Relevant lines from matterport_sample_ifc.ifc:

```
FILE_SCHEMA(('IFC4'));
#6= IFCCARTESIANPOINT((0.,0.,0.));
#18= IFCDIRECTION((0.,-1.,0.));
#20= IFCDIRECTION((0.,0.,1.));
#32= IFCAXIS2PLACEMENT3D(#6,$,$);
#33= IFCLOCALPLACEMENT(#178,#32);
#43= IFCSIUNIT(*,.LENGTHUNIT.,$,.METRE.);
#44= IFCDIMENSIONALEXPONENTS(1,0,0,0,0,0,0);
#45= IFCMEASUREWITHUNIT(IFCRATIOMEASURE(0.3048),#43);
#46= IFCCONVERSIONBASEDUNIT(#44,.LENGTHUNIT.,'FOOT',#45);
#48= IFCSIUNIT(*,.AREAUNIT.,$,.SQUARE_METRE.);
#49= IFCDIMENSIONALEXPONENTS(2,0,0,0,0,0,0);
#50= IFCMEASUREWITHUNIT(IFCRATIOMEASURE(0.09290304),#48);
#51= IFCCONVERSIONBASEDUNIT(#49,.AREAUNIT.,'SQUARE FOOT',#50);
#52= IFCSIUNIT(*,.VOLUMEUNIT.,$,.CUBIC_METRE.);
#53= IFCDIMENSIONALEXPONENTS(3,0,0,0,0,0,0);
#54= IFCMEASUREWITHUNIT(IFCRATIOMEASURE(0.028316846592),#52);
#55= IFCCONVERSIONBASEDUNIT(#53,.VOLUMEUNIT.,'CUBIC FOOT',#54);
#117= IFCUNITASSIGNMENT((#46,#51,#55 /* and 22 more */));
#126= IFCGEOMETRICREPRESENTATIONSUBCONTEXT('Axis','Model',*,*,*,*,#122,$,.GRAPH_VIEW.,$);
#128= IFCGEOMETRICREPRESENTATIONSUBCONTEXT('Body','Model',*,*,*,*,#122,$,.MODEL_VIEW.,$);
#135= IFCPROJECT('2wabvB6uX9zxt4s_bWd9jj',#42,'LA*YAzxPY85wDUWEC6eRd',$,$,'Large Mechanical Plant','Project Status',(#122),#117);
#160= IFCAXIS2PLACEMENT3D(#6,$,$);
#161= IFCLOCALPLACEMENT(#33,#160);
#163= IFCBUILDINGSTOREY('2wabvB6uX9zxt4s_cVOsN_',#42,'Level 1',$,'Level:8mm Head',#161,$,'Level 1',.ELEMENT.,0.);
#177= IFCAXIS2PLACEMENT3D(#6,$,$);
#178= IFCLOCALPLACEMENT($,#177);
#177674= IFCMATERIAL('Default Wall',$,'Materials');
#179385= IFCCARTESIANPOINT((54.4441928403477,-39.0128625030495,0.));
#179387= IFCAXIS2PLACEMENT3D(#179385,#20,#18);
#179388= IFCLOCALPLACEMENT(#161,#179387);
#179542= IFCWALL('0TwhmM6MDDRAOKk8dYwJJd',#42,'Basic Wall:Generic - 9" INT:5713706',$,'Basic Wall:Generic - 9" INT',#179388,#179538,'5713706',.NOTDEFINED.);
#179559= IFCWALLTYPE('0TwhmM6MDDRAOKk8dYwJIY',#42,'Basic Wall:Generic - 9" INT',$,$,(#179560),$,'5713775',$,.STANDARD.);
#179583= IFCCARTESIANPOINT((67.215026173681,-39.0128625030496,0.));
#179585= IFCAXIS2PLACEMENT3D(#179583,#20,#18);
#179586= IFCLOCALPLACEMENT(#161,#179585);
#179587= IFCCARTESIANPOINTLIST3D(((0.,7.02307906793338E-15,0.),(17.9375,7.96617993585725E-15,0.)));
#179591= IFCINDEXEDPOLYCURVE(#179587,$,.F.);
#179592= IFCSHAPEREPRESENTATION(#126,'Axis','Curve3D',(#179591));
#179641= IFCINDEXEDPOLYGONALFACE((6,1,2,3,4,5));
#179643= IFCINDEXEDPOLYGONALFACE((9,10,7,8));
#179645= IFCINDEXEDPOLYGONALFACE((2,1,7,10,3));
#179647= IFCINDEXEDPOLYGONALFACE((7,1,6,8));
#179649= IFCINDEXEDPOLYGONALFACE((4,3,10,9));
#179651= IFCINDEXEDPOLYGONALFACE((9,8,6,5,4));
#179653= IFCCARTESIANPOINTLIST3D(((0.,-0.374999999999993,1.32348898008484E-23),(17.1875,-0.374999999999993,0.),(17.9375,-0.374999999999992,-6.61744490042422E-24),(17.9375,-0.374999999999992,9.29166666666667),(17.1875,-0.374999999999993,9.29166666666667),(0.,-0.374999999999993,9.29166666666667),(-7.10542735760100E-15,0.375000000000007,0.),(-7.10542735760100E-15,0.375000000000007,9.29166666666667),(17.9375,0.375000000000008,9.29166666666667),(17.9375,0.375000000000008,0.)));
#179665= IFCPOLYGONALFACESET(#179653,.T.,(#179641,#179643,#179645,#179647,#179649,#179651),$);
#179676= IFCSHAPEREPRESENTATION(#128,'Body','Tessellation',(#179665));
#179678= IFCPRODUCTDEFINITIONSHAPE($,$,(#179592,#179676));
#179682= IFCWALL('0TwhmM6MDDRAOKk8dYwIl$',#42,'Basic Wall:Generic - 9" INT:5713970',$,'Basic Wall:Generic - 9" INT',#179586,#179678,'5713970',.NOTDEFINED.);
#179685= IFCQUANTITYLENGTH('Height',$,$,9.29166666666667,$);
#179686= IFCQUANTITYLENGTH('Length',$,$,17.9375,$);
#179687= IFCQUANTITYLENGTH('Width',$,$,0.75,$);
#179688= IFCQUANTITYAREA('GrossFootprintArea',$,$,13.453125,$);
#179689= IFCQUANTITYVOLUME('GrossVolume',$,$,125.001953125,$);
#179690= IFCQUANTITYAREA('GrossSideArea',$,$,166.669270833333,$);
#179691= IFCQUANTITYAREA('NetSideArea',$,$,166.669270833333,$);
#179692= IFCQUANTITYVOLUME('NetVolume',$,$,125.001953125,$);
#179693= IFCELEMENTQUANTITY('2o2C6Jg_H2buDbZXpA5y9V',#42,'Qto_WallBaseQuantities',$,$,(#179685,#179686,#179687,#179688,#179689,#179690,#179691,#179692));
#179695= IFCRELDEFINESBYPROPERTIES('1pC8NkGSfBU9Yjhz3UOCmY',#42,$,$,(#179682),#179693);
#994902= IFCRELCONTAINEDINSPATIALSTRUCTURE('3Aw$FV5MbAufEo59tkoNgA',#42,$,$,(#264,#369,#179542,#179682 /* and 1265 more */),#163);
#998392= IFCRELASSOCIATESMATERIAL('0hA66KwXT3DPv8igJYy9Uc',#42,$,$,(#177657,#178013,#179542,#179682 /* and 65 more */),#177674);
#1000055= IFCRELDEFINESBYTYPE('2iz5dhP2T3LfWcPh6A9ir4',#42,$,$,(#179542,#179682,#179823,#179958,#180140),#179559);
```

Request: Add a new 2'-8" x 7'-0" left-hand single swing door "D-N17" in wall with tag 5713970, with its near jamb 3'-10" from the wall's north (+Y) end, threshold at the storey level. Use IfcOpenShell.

```python
import numpy as np
import ifcopenshell
import ifcopenshell.api.feature
import ifcopenshell.api.geometry
import ifcopenshell.api.pset
import ifcopenshell.api.root
import ifcopenshell.api.spatial
import ifcopenshell.geom
import ifcopenshell.util.element
import ifcopenshell.util.placement
import ifcopenshell.util.representation
import ifcopenshell.util.shape
import ifcopenshell.util.unit

model = ifcopenshell.open("matterport_sample_ifc.ifc")
unit_scale = ifcopenshell.util.unit.calculate_unit_scale(model)
area_scale = ifcopenshell.util.unit.calculate_unit_scale(model, "AREAUNIT")
volume_scale = ifcopenshell.util.unit.calculate_unit_scale(model, "VOLUMEUNIT")
settings = ifcopenshell.geom.settings()


def volume(element):
    """Net volume in cubic metres, openings subtracted."""
    shape = ifcopenshell.geom.create_shape(settings, element)
    return ifcopenshell.util.shape.get_volume(shape.geometry)


wall = model.by_guid("0TwhmM6MDDRAOKk8dYwIl$")
storey = ifcopenshell.util.element.get_container(wall, ifc_class="IfcBuildingStorey")
context = ifcopenshell.util.representation.get_context(model, "Model", "Body", "MODEL_VIEW")
before = volume(wall)

width, height, from_end, sill = 0.8128, 2.1336, 1.1684, 0.0  # metres

# The wall runs along its own X axis, and the end named is its -X end.
wall_shape = ifcopenshell.geom.create_shape(settings, wall)
x, y, z = ifcopenshell.util.shape.get_vertices(wall_shape.geometry).T
start = x.min() + from_end
face, thickness = float(y.min()), float(y.max() - y.min())
wall_matrix = ifcopenshell.util.placement.get_local_placement(wall.ObjectPlacement)
level = ifcopenshell.util.placement.get_local_placement(storey.ObjectPlacement)[2, 3]


def in_wall(x, y):
    """Placement at x, y metres in the wall's axes, at sill height."""
    matrix = wall_matrix.copy()
    matrix[:, 3] = wall_matrix @ np.array([x / unit_scale, y / unit_scale, 0.0, 1.0])
    matrix[2, 3] = level + sill / unit_scale
    return matrix


# Opening: a box that overshoots both wall faces by 50 mm.
opening = ifcopenshell.api.root.create_entity(model, ifc_class="IfcOpeningElement", predefined_type="OPENING")
box = ifcopenshell.api.geometry.add_wall_representation(
    model, context=context, length=width, height=height, thickness=thickness + 0.1
)
ifcopenshell.api.geometry.assign_representation(model, product=opening, representation=box)
ifcopenshell.api.geometry.edit_object_placement(model, product=opening, matrix=in_wall(start, face - 0.05), is_si=False)
ifcopenshell.api.feature.add_feature(model, feature=opening, element=wall)

door = ifcopenshell.api.root.create_entity(model, ifc_class="IfcDoor", name="D-N17", predefined_type="DOOR")
door.OverallWidth, door.OverallHeight = width / unit_scale, height / unit_scale
door.OperationType = "SINGLE_SWING_LEFT"
body = ifcopenshell.api.geometry.add_door_representation(
    model,
    context=context,
    overall_width=door.OverallWidth,
    overall_height=door.OverallHeight,
    operation_type="SINGLE_SWING_LEFT",
    lining_properties={"LiningDepth": thickness / unit_scale, "ThresholdDepth": thickness / unit_scale},
)
ifcopenshell.api.geometry.assign_representation(model, product=door, representation=body)
ifcopenshell.api.spatial.assign_container(model, products=[door], relating_structure=storey)
ifcopenshell.api.feature.add_filling(model, opening=opening, element=door)

# The lining spans the wall, so the door starts at the wall face.
ifcopenshell.api.geometry.edit_object_placement(model, product=door, matrix=in_wall(start, face), is_si=False)

after = volume(wall)

# Update the wall's stored quantities.
qto = model.by_id(ifcopenshell.util.element.get_pset(wall, "Qto_WallBaseQuantities", should_inherit=False)["id"])
ifcopenshell.api.pset.edit_qto(model, qto=qto, properties={
    "NetSideArea": after / thickness / area_scale,
    "NetVolume": after / volume_scale,
})

print(f"wall volume {before:.3f} -> {after:.3f} m3")

model.write("matterport_sample_ifc_v2.ifc")
```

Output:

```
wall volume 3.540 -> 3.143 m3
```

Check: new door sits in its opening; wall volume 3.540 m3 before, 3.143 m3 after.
